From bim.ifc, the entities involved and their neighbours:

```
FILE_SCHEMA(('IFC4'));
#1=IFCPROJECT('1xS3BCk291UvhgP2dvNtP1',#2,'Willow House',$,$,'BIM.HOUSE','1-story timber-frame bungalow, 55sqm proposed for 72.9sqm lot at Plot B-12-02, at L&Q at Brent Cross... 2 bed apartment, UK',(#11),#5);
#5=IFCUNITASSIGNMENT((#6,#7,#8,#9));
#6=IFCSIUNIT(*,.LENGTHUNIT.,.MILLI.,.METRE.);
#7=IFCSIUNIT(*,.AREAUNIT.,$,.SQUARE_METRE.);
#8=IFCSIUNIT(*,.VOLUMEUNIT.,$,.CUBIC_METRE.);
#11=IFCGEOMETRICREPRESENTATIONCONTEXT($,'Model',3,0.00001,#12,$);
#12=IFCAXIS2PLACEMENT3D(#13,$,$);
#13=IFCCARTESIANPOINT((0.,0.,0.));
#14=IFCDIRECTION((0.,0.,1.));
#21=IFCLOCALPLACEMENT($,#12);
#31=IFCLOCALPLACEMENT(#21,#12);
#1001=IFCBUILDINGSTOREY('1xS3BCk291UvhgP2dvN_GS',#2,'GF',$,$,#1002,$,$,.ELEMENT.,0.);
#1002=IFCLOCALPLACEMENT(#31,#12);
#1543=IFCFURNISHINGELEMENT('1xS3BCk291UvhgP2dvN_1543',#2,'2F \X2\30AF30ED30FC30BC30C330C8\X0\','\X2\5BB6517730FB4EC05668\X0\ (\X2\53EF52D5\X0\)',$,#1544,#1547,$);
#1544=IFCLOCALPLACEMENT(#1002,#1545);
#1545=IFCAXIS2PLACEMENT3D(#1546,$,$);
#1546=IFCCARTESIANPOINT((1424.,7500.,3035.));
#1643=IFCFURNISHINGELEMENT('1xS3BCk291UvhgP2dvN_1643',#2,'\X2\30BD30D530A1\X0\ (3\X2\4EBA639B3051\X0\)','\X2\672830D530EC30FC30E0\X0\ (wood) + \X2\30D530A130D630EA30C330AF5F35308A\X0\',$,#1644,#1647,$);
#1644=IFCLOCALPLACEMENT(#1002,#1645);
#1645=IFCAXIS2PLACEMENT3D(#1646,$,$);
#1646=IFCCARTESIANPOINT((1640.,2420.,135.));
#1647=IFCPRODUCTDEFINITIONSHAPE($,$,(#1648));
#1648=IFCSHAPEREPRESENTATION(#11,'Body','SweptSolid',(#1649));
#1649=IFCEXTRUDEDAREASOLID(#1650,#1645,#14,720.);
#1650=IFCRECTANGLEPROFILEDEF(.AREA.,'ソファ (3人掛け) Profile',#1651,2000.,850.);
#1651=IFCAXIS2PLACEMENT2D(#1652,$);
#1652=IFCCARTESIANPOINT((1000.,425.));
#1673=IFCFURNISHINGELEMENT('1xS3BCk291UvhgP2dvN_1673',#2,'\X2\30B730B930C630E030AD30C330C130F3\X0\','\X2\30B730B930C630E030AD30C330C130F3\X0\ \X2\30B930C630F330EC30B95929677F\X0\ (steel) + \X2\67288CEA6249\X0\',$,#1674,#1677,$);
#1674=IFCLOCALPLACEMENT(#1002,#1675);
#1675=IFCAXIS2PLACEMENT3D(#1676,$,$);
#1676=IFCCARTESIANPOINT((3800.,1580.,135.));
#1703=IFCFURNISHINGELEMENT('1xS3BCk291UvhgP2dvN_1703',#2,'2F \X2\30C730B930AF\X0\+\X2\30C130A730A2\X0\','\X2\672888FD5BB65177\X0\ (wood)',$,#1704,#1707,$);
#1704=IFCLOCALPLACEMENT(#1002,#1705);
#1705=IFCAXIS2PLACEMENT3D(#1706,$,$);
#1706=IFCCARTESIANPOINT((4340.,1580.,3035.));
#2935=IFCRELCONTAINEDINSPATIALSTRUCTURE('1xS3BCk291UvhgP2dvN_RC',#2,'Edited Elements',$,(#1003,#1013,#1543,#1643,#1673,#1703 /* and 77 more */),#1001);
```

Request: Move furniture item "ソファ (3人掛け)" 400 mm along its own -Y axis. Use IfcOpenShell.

```python
import ifcopenshell
import ifcopenshell.api.geometry
import ifcopenshell.util.placement
import ifcopenshell.util.unit

model = ifcopenshell.open("bim.ifc")
unit_scale = ifcopenshell.util.unit.calculate_unit_scale(model)

item = model.by_id(1643)
matrix = ifcopenshell.util.placement.get_local_placement(item.ObjectPlacement)
matrix[:3, 3] -= matrix[:3, 1] * 0.4 / unit_scale
ifcopenshell.api.geometry.edit_object_placement(model, product=item, matrix=matrix, is_si=False)

print(ifcopenshell.util.placement.get_local_placement(item.ObjectPlacement).round(3) + 0.0)

model.write("bim_updated.ifc")
```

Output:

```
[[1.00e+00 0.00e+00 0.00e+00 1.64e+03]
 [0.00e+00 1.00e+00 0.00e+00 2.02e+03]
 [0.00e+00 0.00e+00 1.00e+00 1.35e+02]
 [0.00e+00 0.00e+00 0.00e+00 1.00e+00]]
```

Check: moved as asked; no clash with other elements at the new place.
